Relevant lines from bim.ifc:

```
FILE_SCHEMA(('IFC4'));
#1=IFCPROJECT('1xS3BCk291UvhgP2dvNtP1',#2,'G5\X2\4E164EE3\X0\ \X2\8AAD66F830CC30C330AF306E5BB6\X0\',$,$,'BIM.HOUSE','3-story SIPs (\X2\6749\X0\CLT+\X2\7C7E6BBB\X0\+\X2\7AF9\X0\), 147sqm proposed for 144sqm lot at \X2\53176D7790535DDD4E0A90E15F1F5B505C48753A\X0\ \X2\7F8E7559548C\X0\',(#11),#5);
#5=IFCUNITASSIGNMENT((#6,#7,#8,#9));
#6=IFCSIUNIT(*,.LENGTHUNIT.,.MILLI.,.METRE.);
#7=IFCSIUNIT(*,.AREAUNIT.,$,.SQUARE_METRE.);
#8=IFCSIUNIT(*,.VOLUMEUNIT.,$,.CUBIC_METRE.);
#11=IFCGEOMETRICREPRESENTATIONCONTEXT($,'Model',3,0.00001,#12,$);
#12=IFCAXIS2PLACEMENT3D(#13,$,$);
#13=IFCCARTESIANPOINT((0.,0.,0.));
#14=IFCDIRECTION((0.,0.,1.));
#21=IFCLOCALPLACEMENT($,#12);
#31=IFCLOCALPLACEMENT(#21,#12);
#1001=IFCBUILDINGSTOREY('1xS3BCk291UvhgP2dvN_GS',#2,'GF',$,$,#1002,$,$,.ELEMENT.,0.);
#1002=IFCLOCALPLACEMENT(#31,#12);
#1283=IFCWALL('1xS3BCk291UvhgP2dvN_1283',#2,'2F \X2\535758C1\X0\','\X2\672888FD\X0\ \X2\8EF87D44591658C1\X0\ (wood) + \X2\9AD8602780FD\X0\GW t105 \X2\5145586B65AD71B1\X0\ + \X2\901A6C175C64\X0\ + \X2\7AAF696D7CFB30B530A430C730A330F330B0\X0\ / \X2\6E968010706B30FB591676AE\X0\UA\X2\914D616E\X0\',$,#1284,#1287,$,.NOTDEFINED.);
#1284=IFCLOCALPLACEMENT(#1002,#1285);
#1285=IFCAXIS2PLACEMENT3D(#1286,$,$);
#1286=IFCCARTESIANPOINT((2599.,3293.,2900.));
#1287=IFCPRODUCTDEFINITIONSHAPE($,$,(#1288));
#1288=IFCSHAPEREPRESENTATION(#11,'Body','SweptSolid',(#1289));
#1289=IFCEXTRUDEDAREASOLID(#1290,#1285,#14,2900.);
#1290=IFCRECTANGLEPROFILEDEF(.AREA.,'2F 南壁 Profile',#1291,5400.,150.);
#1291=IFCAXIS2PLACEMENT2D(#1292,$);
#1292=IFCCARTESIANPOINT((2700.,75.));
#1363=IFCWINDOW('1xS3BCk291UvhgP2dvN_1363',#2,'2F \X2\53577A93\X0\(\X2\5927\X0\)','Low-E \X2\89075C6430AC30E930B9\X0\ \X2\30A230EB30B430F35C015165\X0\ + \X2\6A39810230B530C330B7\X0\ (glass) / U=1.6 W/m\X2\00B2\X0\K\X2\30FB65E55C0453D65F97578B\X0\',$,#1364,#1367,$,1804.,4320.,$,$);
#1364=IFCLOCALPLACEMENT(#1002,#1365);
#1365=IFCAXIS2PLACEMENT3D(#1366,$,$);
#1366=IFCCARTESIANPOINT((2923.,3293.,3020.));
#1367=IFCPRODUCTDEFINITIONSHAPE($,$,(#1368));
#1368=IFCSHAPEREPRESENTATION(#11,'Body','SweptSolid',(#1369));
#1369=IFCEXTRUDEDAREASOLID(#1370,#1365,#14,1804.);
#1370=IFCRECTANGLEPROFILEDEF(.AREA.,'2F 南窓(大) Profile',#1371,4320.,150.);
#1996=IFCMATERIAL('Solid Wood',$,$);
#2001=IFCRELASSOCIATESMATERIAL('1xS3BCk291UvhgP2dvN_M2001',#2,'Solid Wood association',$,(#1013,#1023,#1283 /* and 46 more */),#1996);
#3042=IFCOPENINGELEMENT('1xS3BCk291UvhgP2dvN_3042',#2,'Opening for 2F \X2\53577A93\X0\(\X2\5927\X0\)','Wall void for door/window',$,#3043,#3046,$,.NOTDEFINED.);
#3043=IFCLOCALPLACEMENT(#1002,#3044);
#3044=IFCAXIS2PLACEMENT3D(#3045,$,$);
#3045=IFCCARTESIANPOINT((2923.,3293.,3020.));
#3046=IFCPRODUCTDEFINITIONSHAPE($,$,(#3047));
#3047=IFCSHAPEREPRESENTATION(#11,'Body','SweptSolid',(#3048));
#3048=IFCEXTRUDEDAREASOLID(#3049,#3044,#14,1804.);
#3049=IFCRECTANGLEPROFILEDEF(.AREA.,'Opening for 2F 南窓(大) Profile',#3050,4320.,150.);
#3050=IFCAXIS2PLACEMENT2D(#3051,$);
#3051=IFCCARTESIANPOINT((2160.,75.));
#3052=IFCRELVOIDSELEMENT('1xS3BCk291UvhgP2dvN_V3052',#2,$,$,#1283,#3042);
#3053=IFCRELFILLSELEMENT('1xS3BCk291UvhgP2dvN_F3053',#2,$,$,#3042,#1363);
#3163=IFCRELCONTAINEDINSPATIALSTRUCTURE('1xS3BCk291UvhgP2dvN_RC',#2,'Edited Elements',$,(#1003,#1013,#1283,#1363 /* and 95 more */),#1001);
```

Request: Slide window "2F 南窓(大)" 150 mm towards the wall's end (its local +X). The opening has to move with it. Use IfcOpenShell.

```python
import ifcopenshell
import ifcopenshell.api.geometry
import ifcopenshell.util.placement

model = ifcopenshell.open("bim.ifc")

window = model.by_guid("1xS3BCk291UvhgP2dvN_1363")
opening = window.FillsVoids[0].RelatingOpeningElement
wall = opening.VoidsElements[0].RelatingBuildingElement

wall_matrix = ifcopenshell.util.placement.get_local_placement(wall.ObjectPlacement)
shift = wall_matrix[:3, 0] * 150.0
before = ifcopenshell.util.placement.get_local_placement(window.ObjectPlacement)[:3, 3].copy()

# The window is not placed relative to its opening, so move both.
for product in (opening, window):
    matrix = ifcopenshell.util.placement.get_local_placement(product.ObjectPlacement)
    matrix[:3, 3] += shift
    ifcopenshell.api.geometry.edit_object_placement(model, product=product, matrix=matrix, is_si=False)

after = ifcopenshell.util.placement.get_local_placement(window.ObjectPlacement)[:3, 3]
print("window moved by", (after - before).round(3) + 0.0)

model.write("bim_updated.ifc")
```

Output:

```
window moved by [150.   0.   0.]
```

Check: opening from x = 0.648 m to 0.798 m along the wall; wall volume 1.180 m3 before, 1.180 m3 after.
